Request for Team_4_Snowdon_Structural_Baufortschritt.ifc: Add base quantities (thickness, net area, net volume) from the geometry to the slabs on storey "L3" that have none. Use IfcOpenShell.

First a look at what the model holds.

```python
import ifcopenshell
import ifcopenshell.util.element
import ifcopenshell.util.unit

model = ifcopenshell.open("Team_4_Snowdon_Structural_Baufortschritt.ifc")
print(model.schema)
for unit_type in ("LENGTHUNIT", "AREAUNIT", "VOLUMEUNIT"):
    print(unit_type, ifcopenshell.util.unit.calculate_unit_scale(model, unit_type))
storey = next(s for s in model.by_type("IfcBuildingStorey") if s.Name == "L3")
slabs = [e for e in ifcopenshell.util.element.get_decomposition(storey) if e.is_a("IfcSlab")]
for e in sorted(slabs, key=lambda e: e.id()):
    print(e.id(), e.is_a(), e.Name, list(ifcopenshell.util.element.get_psets(e, qtos_only=True)), sep=" | ")
```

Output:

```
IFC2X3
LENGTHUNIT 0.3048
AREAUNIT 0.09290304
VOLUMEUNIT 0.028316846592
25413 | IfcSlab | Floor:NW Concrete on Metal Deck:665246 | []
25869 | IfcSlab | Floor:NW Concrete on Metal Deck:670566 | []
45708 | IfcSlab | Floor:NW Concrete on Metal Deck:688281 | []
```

```python
import ifcopenshell
import ifcopenshell.api.pset
import ifcopenshell.geom
import ifcopenshell.util.element
import ifcopenshell.util.shape
import ifcopenshell.util.unit

model = ifcopenshell.open("Team_4_Snowdon_Structural_Baufortschritt.ifc")
unit_scale = ifcopenshell.util.unit.calculate_unit_scale(model)
area_scale = ifcopenshell.util.unit.calculate_unit_scale(model, "AREAUNIT")
volume_scale = ifcopenshell.util.unit.calculate_unit_scale(model, "VOLUMEUNIT")
settings = ifcopenshell.geom.settings()

storey = next(s for s in model.by_type("IfcBuildingStorey") if s.Name == "L3")
slabs = [e for e in ifcopenshell.util.element.get_decomposition(storey) if e.is_a("IfcSlab")]

for e in sorted(slabs, key=lambda e: e.id()):
    if ifcopenshell.util.element.get_psets(e, qtos_only=True, should_inherit=False):
        continue
    # Geometry comes back in metres, in the element's own axes.
    shape = ifcopenshell.geom.create_shape(settings, e)
    values = {
        "Width": ifcopenshell.util.shape.get_z(shape.geometry) / unit_scale,
        "NetArea": ifcopenshell.util.shape.get_footprint_area(shape.geometry) / area_scale,
        "NetVolume": ifcopenshell.util.shape.get_volume(shape.geometry) / volume_scale,
    }
    qto = ifcopenshell.api.pset.add_qto(model, product=e, name="BaseQuantities")
    ifcopenshell.api.pset.edit_qto(model, qto=qto, properties=values)
    print(e.id(), {k: round(v, 3) for k, v in values.items()})

model.write("Team_4_Snowdon_Structural_Baufortschritt_updated.ifc")
```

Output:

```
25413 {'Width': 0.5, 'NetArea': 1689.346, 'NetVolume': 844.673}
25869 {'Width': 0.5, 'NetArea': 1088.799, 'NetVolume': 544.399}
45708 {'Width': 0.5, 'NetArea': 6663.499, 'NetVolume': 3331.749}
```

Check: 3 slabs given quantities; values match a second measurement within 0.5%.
